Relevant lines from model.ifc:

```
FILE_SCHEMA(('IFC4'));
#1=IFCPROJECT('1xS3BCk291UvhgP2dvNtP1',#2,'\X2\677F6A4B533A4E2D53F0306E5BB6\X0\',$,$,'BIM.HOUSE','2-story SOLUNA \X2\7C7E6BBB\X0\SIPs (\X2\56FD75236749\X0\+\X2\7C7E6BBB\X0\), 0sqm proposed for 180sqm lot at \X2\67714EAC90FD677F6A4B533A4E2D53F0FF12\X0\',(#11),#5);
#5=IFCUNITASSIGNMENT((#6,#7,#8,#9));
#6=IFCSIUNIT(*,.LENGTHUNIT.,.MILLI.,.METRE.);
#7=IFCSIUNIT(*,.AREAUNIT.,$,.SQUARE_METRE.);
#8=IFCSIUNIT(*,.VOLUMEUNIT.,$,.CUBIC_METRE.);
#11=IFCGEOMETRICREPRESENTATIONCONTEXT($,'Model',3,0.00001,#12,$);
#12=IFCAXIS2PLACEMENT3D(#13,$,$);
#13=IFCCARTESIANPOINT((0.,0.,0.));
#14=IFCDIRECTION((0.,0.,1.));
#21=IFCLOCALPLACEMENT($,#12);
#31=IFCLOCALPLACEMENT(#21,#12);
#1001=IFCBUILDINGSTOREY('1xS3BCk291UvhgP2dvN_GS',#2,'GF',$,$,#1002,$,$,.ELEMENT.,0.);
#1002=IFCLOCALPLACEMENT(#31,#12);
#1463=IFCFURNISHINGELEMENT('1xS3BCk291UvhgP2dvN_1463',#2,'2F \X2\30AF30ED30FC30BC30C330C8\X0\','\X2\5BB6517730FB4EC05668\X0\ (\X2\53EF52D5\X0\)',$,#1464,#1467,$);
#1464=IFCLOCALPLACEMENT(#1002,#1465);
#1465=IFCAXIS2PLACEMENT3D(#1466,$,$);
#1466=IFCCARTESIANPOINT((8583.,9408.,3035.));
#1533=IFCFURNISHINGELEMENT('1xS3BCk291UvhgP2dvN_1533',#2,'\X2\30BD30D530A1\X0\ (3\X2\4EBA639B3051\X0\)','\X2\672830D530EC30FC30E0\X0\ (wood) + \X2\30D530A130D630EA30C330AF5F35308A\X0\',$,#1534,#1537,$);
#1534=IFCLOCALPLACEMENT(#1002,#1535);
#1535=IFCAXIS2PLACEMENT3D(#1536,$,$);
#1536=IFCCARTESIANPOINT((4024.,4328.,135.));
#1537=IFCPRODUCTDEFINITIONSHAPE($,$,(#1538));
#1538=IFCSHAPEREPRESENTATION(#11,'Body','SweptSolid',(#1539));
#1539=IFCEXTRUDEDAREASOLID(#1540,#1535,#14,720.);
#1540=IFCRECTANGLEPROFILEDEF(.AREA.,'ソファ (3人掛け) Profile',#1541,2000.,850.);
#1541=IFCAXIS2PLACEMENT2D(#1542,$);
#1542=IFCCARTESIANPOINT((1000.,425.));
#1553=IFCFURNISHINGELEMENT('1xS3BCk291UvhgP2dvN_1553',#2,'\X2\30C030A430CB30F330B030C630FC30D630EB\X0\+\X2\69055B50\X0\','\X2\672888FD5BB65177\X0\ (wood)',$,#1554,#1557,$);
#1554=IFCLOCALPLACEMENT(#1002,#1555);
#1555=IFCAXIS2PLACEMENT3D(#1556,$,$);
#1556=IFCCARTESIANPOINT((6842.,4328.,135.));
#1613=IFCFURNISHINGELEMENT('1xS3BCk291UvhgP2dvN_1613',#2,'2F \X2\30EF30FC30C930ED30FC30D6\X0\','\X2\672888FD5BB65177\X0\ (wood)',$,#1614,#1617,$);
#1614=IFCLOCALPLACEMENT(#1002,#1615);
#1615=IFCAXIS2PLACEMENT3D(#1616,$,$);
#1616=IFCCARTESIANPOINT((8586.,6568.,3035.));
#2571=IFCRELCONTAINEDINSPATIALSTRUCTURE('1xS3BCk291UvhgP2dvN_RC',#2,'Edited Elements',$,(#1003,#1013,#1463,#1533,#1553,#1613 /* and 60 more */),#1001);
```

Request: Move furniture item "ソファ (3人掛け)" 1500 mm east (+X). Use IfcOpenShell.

```python
import ifcopenshell
import ifcopenshell.api.geometry
import ifcopenshell.util.placement
import ifcopenshell.util.unit

model = ifcopenshell.open("model.ifc")
unit_scale = ifcopenshell.util.unit.calculate_unit_scale(model)

item = model.by_id(1533)
matrix = ifcopenshell.util.placement.get_local_placement(item.ObjectPlacement)
matrix[0, 3] += 1.5 / unit_scale
ifcopenshell.api.geometry.edit_object_placement(model, product=item, matrix=matrix, is_si=False)

print(ifcopenshell.util.placement.get_local_placement(item.ObjectPlacement).round(3) + 0.0)

model.write("model_updated.ifc")
```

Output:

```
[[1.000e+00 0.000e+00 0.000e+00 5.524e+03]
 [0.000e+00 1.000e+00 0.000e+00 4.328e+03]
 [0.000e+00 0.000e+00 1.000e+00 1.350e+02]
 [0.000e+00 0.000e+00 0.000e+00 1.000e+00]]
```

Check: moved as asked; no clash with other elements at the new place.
